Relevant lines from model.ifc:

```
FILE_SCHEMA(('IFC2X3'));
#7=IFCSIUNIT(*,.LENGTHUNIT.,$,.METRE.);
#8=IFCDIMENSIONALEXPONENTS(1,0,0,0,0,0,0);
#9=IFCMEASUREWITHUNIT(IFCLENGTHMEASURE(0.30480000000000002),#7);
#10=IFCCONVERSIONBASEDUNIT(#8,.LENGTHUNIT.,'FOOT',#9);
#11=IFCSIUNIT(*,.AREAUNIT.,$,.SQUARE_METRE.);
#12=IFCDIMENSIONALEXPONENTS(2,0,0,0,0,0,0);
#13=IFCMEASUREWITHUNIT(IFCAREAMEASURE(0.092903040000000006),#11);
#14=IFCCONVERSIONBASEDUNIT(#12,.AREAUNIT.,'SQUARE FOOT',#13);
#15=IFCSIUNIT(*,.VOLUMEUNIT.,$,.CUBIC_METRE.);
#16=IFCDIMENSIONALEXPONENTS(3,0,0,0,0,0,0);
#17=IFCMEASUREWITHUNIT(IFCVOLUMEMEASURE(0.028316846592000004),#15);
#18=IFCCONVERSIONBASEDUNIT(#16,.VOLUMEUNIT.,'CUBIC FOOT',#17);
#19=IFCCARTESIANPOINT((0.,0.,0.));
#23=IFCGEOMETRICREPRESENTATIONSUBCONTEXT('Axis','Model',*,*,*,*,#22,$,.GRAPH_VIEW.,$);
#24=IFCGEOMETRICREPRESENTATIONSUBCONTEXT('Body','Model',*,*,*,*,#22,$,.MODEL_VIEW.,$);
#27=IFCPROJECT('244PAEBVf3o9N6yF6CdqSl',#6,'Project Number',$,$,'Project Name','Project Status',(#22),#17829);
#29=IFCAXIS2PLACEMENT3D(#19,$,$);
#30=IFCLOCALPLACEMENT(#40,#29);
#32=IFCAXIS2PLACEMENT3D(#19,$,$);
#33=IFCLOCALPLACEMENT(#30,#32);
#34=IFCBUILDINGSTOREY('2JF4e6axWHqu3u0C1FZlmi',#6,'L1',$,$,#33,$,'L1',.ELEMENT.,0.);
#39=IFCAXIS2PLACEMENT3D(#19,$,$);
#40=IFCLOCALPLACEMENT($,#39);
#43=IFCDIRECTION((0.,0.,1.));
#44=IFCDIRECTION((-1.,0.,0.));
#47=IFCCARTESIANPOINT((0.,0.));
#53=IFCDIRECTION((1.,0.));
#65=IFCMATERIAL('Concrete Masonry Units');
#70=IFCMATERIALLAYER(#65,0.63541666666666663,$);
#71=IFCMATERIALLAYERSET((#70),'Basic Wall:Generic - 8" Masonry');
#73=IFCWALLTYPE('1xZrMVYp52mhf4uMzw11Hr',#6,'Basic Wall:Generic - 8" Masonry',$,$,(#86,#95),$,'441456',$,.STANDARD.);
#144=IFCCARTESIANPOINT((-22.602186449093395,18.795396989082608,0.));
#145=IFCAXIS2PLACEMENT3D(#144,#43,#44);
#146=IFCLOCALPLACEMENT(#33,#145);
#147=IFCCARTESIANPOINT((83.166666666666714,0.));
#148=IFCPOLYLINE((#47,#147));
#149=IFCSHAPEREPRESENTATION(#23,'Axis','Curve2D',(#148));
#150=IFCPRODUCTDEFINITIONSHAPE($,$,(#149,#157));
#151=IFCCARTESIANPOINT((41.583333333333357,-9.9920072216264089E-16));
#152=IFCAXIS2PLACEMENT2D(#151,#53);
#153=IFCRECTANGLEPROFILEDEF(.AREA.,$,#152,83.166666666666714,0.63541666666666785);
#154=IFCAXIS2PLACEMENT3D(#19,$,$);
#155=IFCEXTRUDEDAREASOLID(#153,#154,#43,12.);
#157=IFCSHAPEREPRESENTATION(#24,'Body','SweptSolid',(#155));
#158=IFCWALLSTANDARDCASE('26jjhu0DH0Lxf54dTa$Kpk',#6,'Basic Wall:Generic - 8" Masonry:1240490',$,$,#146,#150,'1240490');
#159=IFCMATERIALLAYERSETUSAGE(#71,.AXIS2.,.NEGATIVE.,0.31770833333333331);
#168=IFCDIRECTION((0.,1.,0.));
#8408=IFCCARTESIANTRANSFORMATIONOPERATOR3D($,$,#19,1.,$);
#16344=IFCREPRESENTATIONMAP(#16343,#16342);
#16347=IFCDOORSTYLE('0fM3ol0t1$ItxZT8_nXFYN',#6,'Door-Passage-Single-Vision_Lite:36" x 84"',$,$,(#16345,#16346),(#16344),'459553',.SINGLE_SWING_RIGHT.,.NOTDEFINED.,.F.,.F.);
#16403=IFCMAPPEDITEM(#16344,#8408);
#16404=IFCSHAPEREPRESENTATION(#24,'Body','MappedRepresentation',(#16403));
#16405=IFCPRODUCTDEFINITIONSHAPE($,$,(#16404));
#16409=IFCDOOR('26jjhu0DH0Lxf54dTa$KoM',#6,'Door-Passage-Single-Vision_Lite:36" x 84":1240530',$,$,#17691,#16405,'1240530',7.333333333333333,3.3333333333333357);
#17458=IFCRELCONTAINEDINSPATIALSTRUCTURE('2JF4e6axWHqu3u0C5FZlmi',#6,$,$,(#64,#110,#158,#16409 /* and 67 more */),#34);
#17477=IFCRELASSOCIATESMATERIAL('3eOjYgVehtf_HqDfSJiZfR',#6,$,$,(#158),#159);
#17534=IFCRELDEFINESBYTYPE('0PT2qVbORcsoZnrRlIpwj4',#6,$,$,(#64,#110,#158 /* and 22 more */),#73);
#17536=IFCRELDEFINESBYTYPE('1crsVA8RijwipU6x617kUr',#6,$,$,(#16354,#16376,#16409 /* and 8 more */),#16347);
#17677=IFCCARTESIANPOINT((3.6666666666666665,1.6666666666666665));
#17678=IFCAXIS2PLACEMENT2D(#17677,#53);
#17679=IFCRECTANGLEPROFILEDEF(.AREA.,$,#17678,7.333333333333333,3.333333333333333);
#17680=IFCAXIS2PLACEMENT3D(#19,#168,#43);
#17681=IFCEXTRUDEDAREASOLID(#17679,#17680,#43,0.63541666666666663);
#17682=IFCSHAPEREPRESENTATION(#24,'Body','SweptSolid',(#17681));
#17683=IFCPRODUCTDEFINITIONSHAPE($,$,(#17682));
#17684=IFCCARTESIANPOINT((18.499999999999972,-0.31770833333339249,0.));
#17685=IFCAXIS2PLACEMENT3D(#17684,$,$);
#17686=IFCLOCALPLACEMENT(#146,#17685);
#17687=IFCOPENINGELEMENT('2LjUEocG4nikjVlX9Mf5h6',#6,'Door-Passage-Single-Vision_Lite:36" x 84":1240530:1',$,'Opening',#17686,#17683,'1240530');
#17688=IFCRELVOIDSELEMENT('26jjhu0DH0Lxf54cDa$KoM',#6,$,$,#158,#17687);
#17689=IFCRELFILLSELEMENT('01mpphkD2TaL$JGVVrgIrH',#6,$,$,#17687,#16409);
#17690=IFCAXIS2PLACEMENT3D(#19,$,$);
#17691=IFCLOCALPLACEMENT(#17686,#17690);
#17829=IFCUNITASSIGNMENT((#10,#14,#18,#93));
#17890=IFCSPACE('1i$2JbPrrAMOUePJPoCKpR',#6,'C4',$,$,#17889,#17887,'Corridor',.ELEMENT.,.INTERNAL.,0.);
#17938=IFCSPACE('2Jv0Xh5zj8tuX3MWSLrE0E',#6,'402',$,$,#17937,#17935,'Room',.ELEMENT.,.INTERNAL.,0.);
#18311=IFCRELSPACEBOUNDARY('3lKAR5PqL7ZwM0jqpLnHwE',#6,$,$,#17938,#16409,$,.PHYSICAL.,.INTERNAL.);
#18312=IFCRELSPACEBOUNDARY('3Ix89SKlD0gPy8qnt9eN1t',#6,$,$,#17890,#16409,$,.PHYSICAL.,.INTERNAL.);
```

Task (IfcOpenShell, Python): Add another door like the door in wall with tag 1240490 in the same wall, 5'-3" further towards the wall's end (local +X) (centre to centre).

```python
import ifcopenshell
import ifcopenshell.api.feature
import ifcopenshell.api.geometry
import ifcopenshell.api.root
import ifcopenshell.geom
import ifcopenshell.util.element
import ifcopenshell.util.placement
import ifcopenshell.util.shape
import ifcopenshell.util.unit

model = ifcopenshell.open("model.ifc")
unit_scale = ifcopenshell.util.unit.calculate_unit_scale(model)
settings = ifcopenshell.geom.settings()


def volume(element):
    """Net volume in cubic metres, openings subtracted."""
    shape = ifcopenshell.geom.create_shape(settings, element)
    return ifcopenshell.util.shape.get_volume(shape.geometry)


def reuse_history(source, copy):
    """copy_class also copies each property set's owner history, people and application; keep the originals."""
    for rel in copy.IsDefinedBy:
        if rel.is_a("IfcRelDefinesByProperties") and (history := rel.RelatingPropertyDefinition.OwnerHistory):
            rel.RelatingPropertyDefinition.OwnerHistory = source.OwnerHistory
            ifcopenshell.util.element.remove_deep2(model, history)


door = model.by_guid("26jjhu0DH0Lxf54dTa$KoM")
opening = door.FillsVoids[0].RelatingOpeningElement
wall = opening.VoidsElements[0].RelatingBuildingElement
before = volume(wall)
shift = ifcopenshell.util.placement.get_local_placement(wall.ObjectPlacement)[:3, 0] * 63 * 0.0254 / unit_scale

# copy_class copies the void relationship, type, container and properties, but no geometry.
new_opening = ifcopenshell.api.root.copy_class(model, product=opening)
new_opening.Representation = ifcopenshell.util.element.copy_deep(
    model, opening.Representation, exclude=["IfcGeometricRepresentationContext", "IfcRepresentationMap"]
)
new_opening.Name = 'Door-Passage-Single-Vision_Lite:36" x 84"'
new_opening.Tag = None
new_door = ifcopenshell.api.root.copy_class(model, product=door)
new_door.Representation = ifcopenshell.util.element.copy_deep(
    model, door.Representation, exclude=["IfcGeometricRepresentationContext", "IfcRepresentationMap"]
)
new_door.Name = 'Door-Passage-Single-Vision_Lite:36" x 84"'
new_door.Tag = None
reuse_history(door, new_door)
fills = ifcopenshell.api.feature.add_filling(model, opening=new_opening, element=new_door)
fills.OwnerHistory = new_door.OwnerHistory  # required in IFC2X3

for old, new in ((opening, new_opening), (door, new_door)):
    matrix = ifcopenshell.util.placement.get_local_placement(old.ObjectPlacement)
    matrix[:3, 3] += shift
    ifcopenshell.api.geometry.edit_object_placement(model, product=new, matrix=matrix, is_si=False)

after = volume(wall)

print(f"wall volume {before:.3f} -> {after:.3f} m3")

model.write("model_edited.ifc")
```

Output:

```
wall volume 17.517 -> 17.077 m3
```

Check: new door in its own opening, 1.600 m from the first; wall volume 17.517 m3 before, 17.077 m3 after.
